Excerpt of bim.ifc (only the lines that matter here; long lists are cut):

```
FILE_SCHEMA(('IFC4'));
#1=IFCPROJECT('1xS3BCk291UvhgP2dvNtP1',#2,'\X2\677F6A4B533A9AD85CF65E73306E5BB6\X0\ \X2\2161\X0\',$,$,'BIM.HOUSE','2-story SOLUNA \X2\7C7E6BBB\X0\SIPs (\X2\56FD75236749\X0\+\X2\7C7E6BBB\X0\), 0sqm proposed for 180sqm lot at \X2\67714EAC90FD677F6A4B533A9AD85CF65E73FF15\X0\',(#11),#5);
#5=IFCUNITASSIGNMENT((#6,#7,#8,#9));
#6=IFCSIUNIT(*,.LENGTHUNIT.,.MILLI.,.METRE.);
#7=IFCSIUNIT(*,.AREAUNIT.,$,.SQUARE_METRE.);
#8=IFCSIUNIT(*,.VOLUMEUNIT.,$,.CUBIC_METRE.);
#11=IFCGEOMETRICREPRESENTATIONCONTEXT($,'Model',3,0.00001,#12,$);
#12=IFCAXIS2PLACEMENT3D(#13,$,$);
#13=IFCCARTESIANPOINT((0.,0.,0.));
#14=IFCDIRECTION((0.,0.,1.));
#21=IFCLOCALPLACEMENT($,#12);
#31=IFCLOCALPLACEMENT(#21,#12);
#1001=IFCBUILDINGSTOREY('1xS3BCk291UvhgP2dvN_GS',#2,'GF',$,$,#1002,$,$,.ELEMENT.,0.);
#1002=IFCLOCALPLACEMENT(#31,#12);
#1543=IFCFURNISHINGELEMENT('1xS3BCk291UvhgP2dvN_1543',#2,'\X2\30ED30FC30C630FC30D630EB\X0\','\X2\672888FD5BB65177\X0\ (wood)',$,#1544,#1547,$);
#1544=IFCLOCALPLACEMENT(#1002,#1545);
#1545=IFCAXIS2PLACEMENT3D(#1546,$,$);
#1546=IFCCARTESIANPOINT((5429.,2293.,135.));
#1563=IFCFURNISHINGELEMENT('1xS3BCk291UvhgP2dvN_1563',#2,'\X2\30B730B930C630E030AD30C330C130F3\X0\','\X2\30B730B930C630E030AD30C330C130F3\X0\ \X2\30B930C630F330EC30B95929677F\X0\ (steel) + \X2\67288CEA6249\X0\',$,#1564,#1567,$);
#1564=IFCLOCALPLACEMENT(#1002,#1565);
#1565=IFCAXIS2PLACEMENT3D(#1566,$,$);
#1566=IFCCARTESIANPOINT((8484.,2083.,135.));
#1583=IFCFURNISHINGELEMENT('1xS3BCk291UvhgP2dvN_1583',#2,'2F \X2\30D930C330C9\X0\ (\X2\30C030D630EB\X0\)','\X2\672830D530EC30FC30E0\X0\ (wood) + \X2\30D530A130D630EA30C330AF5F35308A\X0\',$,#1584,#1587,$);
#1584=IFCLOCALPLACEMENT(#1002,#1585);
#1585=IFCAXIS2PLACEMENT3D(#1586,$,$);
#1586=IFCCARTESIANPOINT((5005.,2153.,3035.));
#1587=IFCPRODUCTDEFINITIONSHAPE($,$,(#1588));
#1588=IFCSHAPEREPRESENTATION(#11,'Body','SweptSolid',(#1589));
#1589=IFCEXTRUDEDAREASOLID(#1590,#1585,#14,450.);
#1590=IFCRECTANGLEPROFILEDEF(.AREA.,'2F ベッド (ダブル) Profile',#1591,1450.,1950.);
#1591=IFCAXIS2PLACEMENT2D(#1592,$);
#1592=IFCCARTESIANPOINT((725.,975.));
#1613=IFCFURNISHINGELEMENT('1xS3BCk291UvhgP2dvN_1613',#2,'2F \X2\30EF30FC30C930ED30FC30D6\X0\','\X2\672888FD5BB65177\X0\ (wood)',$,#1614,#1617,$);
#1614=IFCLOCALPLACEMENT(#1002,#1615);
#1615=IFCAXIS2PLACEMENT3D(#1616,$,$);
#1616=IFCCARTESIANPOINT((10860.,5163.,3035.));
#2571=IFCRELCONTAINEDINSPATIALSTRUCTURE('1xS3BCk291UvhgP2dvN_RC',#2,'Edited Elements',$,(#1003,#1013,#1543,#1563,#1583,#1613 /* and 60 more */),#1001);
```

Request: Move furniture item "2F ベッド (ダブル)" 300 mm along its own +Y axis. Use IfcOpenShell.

```python
import ifcopenshell
import ifcopenshell.api.geometry
import ifcopenshell.util.placement
import ifcopenshell.util.unit

model = ifcopenshell.open("bim.ifc")
unit_scale = ifcopenshell.util.unit.calculate_unit_scale(model)

item = model.by_guid("1xS3BCk291UvhgP2dvN_1583")
matrix = ifcopenshell.util.placement.get_local_placement(item.ObjectPlacement)
matrix[:3, 3] += matrix[:3, 1] * 0.3 / unit_scale
ifcopenshell.api.geometry.edit_object_placement(model, product=item, matrix=matrix, is_si=False)

print(ifcopenshell.util.placement.get_local_placement(item.ObjectPlacement).round(3) + 0.0)

model.write("bim_rev.ifc")
```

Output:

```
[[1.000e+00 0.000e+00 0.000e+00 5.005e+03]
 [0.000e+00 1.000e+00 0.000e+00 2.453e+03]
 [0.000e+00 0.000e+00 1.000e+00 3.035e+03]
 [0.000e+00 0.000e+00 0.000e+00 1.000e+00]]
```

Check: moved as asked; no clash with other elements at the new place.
